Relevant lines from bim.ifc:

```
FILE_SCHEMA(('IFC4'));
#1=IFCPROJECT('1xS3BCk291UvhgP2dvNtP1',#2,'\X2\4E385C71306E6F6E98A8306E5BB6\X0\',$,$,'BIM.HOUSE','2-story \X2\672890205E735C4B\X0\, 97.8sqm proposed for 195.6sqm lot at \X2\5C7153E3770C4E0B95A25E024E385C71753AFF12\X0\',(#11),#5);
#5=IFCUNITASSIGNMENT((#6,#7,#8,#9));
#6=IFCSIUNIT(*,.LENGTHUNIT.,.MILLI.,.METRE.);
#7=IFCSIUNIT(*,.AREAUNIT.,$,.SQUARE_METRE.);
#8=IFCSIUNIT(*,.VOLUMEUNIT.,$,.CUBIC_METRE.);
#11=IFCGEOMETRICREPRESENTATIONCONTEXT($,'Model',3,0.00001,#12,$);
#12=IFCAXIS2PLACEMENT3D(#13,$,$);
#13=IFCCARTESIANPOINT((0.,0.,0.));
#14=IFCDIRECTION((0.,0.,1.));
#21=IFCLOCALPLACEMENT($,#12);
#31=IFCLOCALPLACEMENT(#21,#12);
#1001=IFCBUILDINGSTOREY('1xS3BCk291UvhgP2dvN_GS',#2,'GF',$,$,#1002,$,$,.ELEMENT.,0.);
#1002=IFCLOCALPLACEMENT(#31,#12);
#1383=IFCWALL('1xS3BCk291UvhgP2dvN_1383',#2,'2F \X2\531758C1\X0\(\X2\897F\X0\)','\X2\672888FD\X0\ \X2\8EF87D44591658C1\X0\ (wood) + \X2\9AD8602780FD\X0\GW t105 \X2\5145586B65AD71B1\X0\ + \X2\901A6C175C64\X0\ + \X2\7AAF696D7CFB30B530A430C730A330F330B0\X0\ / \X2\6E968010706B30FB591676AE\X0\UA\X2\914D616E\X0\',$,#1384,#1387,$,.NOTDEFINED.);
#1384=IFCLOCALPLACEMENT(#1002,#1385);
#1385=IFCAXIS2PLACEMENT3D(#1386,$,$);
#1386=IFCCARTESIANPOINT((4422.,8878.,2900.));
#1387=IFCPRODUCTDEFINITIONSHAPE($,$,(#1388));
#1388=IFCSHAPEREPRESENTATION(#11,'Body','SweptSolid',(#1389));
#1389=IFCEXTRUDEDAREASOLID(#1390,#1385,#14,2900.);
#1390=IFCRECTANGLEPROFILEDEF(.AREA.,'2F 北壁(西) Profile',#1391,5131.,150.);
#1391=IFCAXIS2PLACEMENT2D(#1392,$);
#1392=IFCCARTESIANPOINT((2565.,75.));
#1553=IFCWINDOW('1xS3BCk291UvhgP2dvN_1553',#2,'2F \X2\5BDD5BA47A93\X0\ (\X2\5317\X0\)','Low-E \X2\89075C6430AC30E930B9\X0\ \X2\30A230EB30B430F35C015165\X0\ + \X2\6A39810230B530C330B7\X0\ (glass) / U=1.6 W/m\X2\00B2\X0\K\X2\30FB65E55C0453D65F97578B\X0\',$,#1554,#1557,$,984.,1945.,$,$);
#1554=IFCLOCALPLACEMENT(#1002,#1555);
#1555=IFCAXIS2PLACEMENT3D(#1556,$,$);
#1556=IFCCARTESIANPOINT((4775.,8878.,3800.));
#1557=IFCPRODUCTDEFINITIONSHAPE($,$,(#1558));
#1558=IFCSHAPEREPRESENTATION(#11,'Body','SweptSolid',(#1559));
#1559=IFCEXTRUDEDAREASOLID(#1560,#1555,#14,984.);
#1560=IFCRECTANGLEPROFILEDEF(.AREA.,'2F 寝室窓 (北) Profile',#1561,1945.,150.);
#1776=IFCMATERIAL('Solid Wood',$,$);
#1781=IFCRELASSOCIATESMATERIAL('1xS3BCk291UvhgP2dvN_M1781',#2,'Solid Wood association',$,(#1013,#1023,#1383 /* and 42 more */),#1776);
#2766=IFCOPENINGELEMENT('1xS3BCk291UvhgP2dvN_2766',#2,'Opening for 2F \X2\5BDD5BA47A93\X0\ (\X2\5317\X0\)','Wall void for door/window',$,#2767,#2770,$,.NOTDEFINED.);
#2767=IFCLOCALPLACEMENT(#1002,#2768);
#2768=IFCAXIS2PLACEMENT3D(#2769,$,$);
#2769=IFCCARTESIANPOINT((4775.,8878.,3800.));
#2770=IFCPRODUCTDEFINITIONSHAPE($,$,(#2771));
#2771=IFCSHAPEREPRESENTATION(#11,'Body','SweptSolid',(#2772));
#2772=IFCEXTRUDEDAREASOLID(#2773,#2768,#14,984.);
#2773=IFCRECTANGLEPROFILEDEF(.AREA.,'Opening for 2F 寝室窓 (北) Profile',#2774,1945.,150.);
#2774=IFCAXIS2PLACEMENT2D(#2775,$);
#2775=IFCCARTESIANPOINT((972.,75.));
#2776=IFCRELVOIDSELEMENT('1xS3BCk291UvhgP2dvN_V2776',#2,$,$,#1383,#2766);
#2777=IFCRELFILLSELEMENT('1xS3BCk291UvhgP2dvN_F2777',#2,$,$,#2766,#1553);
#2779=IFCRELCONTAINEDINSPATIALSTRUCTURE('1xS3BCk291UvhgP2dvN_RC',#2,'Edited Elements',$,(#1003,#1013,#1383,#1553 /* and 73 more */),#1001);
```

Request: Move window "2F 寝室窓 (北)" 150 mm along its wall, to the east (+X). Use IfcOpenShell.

```python
import ifcopenshell
import ifcopenshell.api.geometry
import ifcopenshell.util.placement
import ifcopenshell.util.unit

model = ifcopenshell.open("bim.ifc")
unit_scale = ifcopenshell.util.unit.calculate_unit_scale(model)

window = model.by_guid("1xS3BCk291UvhgP2dvN_1553")
opening = window.FillsVoids[0].RelatingOpeningElement
wall = opening.VoidsElements[0].RelatingBuildingElement

wall_matrix = ifcopenshell.util.placement.get_local_placement(wall.ObjectPlacement)
shift = wall_matrix[:3, 0] * 0.15 / unit_scale
before = ifcopenshell.util.placement.get_local_placement(window.ObjectPlacement)[:3, 3].copy()

# The window is not placed relative to its opening, so move both.
for product in (opening, window):
    matrix = ifcopenshell.util.placement.get_local_placement(product.ObjectPlacement)
    matrix[:3, 3] += shift
    ifcopenshell.api.geometry.edit_object_placement(model, product=product, matrix=matrix, is_si=False)

after = ifcopenshell.util.placement.get_local_placement(window.ObjectPlacement)[:3, 3]
print("window moved by", (after - before).round(3) + 0.0)

model.write("bim_v2.ifc")
```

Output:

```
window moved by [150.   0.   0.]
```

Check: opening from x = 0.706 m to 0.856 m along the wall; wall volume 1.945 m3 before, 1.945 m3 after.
